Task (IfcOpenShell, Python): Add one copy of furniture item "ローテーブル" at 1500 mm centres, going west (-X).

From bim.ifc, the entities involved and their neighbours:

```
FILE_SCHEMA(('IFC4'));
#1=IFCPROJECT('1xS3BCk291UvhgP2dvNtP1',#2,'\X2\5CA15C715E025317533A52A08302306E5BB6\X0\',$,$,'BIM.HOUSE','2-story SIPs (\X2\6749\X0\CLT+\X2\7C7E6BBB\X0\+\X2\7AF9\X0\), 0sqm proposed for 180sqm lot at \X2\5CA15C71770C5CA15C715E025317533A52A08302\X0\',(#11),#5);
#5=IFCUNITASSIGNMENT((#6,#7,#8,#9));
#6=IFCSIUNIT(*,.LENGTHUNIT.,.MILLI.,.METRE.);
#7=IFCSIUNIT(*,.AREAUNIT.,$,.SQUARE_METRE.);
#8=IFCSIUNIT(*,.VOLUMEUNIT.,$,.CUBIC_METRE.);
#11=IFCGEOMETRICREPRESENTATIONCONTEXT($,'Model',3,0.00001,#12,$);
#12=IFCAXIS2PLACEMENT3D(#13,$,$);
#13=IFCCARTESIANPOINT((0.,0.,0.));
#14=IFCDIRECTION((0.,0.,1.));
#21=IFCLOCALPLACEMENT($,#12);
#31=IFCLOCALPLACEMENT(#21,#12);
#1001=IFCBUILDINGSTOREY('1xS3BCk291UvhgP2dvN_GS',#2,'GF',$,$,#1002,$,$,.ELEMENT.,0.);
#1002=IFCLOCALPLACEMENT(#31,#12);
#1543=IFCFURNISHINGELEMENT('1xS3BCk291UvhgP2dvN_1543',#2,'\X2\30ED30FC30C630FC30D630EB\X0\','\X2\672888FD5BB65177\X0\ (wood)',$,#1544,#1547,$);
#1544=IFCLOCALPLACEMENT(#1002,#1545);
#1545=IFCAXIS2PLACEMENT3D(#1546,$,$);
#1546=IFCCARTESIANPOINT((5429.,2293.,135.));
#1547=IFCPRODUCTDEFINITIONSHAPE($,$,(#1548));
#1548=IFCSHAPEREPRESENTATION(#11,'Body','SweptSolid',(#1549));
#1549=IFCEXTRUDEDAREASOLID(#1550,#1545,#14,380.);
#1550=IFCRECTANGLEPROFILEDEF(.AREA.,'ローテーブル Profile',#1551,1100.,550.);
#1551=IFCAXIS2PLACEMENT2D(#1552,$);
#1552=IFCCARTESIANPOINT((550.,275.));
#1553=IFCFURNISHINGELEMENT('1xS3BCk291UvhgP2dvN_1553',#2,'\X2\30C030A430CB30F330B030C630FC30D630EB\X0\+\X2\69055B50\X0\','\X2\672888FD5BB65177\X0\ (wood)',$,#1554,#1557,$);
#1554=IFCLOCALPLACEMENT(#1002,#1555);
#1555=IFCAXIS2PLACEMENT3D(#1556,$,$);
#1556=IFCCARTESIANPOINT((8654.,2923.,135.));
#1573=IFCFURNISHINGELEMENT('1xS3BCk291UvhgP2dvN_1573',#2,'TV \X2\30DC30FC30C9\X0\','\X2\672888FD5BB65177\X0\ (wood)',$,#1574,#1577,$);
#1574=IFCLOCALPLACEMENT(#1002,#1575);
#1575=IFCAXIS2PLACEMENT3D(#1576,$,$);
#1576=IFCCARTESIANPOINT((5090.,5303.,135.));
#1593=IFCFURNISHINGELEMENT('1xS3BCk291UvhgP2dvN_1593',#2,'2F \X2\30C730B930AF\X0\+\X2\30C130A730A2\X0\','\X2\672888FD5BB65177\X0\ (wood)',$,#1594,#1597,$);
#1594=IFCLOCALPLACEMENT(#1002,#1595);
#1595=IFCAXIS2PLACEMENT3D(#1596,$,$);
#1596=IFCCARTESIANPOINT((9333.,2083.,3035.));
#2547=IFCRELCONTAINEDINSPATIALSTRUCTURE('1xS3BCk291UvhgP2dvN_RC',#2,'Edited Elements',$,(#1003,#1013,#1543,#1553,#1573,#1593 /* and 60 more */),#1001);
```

```python
import numpy as np
import ifcopenshell
import ifcopenshell.api.geometry
import ifcopenshell.api.root
import ifcopenshell.util.element
import ifcopenshell.util.placement
import ifcopenshell.util.unit

model = ifcopenshell.open("bim.ifc")
unit_scale = ifcopenshell.util.unit.calculate_unit_scale(model)


def reuse_history(source, copy):
    """copy_class also copies each property set's owner history, people and application; keep the originals."""
    for rel in copy.IsDefinedBy:
        if rel.is_a("IfcRelDefinesByProperties") and (history := rel.RelatingPropertyDefinition.OwnerHistory):
            rel.RelatingPropertyDefinition.OwnerHistory = source.OwnerHistory
            ifcopenshell.util.element.remove_deep2(model, history)


source = model.by_guid("1xS3BCk291UvhgP2dvN_1543")
base = ifcopenshell.util.placement.get_local_placement(source.ObjectPlacement)
step = np.array([-1.0, 0.0, 0.0]) * 1.5 / unit_scale

for i in range(1, 2):
    copy = ifcopenshell.api.root.copy_class(model, product=source)
    copy.Representation = ifcopenshell.util.element.copy_deep(
        model, source.Representation, exclude=["IfcGeometricRepresentationContext", "IfcRepresentationMap"]
    )
    reuse_history(source, copy)
    matrix = base.copy()
    matrix[:3, 3] += i * step
    print("added at", matrix[:3, 3].round(3) + 0.0)
    ifcopenshell.api.geometry.edit_object_placement(model, product=copy, matrix=matrix, is_si=False)

model.write("bim_updated.ifc")
```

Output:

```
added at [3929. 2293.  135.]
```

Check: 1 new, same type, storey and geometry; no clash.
